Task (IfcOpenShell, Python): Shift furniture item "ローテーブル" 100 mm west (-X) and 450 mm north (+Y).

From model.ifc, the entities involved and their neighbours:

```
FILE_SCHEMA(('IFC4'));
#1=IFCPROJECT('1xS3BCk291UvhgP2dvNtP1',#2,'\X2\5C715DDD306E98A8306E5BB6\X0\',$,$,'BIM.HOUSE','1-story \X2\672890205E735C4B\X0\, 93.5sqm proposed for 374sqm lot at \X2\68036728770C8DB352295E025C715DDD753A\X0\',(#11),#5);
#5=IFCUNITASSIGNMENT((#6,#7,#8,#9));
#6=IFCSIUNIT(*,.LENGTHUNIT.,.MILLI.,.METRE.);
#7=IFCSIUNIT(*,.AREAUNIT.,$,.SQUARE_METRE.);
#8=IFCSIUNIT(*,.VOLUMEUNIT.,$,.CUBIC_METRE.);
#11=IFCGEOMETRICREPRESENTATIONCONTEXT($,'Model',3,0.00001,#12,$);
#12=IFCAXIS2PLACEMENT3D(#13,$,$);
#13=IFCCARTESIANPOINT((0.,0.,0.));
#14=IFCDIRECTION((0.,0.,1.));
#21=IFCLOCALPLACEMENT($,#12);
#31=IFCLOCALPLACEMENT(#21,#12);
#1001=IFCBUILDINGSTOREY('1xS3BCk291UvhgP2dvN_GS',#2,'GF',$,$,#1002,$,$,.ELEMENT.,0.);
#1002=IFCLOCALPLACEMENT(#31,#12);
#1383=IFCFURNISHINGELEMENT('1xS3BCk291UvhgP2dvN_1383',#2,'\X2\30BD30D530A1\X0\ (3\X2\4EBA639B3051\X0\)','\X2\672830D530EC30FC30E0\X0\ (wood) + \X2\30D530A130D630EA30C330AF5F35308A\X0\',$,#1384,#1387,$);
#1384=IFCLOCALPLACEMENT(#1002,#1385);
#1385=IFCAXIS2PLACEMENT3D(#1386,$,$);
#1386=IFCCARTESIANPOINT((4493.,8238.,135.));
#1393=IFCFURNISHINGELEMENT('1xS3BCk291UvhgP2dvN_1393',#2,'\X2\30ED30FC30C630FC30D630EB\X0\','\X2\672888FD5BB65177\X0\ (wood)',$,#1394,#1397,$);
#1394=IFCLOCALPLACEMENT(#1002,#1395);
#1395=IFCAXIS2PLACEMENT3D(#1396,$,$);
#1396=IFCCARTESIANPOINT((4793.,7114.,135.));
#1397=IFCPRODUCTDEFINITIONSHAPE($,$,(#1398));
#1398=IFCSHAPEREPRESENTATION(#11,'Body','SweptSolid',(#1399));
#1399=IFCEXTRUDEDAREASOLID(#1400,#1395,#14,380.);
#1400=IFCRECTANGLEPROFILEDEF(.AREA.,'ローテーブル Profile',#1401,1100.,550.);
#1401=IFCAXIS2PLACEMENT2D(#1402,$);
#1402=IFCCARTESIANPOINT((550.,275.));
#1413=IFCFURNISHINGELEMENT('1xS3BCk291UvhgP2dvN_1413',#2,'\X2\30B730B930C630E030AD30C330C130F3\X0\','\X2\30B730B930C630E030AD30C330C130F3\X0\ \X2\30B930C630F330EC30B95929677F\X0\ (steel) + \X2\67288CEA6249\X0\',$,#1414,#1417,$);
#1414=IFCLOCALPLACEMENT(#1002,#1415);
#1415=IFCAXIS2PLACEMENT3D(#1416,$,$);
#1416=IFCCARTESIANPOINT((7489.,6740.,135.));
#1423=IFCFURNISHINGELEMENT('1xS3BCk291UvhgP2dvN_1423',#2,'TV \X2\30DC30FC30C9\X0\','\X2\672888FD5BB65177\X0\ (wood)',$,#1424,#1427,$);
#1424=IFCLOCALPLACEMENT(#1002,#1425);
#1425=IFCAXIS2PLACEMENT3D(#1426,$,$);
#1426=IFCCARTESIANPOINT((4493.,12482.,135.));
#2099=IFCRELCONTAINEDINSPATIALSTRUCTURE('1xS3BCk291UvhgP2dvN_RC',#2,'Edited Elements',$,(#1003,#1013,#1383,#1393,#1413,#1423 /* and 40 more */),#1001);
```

```python
import ifcopenshell
import ifcopenshell.api.geometry
import ifcopenshell.util.placement
import ifcopenshell.util.unit

model = ifcopenshell.open("model.ifc")
unit_scale = ifcopenshell.util.unit.calculate_unit_scale(model)

item = model.by_guid("1xS3BCk291UvhgP2dvN_1393")
matrix = ifcopenshell.util.placement.get_local_placement(item.ObjectPlacement)
matrix[0, 3] -= 0.1 / unit_scale
matrix[1, 3] += 0.45 / unit_scale
ifcopenshell.api.geometry.edit_object_placement(model, product=item, matrix=matrix, is_si=False)

print(ifcopenshell.util.placement.get_local_placement(item.ObjectPlacement).round(3) + 0.0)

model.write("model_v2.ifc")
```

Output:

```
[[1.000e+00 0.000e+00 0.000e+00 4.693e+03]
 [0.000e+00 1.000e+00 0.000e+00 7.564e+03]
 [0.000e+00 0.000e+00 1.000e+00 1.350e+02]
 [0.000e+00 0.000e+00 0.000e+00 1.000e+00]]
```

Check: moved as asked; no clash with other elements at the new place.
